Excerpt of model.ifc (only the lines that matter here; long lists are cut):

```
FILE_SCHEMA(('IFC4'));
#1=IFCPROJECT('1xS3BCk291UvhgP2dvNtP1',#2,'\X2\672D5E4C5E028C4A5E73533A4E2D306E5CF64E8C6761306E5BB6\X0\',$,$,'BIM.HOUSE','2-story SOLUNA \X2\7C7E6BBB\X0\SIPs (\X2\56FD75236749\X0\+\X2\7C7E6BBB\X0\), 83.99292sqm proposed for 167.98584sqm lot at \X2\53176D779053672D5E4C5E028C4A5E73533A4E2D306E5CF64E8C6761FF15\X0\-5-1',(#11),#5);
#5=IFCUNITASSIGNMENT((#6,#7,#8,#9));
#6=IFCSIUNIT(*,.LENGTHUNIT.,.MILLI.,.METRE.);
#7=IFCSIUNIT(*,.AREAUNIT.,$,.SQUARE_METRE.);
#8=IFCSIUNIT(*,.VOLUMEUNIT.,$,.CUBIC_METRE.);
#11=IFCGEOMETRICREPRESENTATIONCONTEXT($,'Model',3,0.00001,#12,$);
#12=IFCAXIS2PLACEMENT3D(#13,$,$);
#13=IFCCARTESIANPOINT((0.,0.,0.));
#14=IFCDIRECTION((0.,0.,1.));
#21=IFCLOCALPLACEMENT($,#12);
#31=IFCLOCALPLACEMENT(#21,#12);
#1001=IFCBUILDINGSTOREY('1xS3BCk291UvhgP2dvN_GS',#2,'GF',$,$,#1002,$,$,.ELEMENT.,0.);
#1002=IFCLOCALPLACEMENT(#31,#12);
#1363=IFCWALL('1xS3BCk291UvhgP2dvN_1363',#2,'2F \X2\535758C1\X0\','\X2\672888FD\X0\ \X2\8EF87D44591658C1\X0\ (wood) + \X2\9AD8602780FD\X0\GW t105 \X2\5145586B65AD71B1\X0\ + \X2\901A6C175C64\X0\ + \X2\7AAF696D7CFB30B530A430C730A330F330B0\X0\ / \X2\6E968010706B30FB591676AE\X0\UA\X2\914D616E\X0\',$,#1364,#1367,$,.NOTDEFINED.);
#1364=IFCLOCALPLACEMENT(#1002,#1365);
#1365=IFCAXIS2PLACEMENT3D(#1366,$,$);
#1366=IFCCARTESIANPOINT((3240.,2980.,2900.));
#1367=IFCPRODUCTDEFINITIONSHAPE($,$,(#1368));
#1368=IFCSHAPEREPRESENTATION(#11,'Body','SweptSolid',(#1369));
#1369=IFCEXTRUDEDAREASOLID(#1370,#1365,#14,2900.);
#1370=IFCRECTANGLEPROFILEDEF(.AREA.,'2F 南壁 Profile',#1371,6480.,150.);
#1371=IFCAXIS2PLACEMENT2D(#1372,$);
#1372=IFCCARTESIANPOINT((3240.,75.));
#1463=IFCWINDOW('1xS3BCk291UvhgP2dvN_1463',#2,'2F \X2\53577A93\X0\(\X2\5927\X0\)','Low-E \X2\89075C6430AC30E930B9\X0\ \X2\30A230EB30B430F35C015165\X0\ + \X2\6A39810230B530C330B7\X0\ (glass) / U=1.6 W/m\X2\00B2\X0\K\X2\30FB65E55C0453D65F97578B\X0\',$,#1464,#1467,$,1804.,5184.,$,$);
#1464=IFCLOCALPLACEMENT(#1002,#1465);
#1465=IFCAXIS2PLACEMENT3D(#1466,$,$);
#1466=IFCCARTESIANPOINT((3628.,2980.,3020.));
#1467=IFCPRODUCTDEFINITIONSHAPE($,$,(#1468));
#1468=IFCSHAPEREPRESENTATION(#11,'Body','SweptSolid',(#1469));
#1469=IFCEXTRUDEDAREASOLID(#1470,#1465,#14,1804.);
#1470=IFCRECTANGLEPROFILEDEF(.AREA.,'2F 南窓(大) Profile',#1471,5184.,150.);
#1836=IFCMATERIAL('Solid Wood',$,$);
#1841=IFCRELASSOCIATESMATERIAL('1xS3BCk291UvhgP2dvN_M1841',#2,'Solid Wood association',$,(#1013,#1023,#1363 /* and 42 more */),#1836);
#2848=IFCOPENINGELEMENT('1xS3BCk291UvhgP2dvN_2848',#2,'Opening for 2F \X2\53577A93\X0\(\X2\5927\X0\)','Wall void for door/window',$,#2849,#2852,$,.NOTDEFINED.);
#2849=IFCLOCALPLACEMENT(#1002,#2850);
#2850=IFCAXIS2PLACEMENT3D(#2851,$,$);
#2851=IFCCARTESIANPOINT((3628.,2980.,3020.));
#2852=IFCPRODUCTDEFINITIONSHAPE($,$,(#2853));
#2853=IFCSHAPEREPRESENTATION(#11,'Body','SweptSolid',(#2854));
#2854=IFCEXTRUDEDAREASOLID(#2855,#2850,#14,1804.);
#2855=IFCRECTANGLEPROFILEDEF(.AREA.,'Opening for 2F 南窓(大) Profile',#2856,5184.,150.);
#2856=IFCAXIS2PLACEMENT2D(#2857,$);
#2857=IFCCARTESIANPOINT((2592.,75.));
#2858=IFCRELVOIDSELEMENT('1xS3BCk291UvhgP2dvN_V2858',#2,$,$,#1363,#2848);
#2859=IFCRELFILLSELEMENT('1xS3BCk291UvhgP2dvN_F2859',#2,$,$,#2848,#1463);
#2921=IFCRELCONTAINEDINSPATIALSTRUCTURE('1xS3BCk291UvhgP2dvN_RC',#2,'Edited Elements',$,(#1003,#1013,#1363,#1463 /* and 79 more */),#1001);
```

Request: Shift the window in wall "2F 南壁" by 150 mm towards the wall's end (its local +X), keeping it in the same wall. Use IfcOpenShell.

```python
import ifcopenshell
import ifcopenshell.api.geometry
import ifcopenshell.util.placement

model = ifcopenshell.open("model.ifc")

window = model.by_id(1463)
opening = window.FillsVoids[0].RelatingOpeningElement
wall = opening.VoidsElements[0].RelatingBuildingElement

wall_matrix = ifcopenshell.util.placement.get_local_placement(wall.ObjectPlacement)
shift = wall_matrix[:3, 0] * 150.0
before = ifcopenshell.util.placement.get_local_placement(window.ObjectPlacement)[:3, 3].copy()

# The window is not placed relative to its opening, so move both.
for product in (opening, window):
    matrix = ifcopenshell.util.placement.get_local_placement(product.ObjectPlacement)
    matrix[:3, 3] += shift
    ifcopenshell.api.geometry.edit_object_placement(model, product=product, matrix=matrix, is_si=False)

after = ifcopenshell.util.placement.get_local_placement(window.ObjectPlacement)[:3, 3]
print("window moved by", (after - before).round(3) + 0.0)

model.write("model_updated.ifc")
```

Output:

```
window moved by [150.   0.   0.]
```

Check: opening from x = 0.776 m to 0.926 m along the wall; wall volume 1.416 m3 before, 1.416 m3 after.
